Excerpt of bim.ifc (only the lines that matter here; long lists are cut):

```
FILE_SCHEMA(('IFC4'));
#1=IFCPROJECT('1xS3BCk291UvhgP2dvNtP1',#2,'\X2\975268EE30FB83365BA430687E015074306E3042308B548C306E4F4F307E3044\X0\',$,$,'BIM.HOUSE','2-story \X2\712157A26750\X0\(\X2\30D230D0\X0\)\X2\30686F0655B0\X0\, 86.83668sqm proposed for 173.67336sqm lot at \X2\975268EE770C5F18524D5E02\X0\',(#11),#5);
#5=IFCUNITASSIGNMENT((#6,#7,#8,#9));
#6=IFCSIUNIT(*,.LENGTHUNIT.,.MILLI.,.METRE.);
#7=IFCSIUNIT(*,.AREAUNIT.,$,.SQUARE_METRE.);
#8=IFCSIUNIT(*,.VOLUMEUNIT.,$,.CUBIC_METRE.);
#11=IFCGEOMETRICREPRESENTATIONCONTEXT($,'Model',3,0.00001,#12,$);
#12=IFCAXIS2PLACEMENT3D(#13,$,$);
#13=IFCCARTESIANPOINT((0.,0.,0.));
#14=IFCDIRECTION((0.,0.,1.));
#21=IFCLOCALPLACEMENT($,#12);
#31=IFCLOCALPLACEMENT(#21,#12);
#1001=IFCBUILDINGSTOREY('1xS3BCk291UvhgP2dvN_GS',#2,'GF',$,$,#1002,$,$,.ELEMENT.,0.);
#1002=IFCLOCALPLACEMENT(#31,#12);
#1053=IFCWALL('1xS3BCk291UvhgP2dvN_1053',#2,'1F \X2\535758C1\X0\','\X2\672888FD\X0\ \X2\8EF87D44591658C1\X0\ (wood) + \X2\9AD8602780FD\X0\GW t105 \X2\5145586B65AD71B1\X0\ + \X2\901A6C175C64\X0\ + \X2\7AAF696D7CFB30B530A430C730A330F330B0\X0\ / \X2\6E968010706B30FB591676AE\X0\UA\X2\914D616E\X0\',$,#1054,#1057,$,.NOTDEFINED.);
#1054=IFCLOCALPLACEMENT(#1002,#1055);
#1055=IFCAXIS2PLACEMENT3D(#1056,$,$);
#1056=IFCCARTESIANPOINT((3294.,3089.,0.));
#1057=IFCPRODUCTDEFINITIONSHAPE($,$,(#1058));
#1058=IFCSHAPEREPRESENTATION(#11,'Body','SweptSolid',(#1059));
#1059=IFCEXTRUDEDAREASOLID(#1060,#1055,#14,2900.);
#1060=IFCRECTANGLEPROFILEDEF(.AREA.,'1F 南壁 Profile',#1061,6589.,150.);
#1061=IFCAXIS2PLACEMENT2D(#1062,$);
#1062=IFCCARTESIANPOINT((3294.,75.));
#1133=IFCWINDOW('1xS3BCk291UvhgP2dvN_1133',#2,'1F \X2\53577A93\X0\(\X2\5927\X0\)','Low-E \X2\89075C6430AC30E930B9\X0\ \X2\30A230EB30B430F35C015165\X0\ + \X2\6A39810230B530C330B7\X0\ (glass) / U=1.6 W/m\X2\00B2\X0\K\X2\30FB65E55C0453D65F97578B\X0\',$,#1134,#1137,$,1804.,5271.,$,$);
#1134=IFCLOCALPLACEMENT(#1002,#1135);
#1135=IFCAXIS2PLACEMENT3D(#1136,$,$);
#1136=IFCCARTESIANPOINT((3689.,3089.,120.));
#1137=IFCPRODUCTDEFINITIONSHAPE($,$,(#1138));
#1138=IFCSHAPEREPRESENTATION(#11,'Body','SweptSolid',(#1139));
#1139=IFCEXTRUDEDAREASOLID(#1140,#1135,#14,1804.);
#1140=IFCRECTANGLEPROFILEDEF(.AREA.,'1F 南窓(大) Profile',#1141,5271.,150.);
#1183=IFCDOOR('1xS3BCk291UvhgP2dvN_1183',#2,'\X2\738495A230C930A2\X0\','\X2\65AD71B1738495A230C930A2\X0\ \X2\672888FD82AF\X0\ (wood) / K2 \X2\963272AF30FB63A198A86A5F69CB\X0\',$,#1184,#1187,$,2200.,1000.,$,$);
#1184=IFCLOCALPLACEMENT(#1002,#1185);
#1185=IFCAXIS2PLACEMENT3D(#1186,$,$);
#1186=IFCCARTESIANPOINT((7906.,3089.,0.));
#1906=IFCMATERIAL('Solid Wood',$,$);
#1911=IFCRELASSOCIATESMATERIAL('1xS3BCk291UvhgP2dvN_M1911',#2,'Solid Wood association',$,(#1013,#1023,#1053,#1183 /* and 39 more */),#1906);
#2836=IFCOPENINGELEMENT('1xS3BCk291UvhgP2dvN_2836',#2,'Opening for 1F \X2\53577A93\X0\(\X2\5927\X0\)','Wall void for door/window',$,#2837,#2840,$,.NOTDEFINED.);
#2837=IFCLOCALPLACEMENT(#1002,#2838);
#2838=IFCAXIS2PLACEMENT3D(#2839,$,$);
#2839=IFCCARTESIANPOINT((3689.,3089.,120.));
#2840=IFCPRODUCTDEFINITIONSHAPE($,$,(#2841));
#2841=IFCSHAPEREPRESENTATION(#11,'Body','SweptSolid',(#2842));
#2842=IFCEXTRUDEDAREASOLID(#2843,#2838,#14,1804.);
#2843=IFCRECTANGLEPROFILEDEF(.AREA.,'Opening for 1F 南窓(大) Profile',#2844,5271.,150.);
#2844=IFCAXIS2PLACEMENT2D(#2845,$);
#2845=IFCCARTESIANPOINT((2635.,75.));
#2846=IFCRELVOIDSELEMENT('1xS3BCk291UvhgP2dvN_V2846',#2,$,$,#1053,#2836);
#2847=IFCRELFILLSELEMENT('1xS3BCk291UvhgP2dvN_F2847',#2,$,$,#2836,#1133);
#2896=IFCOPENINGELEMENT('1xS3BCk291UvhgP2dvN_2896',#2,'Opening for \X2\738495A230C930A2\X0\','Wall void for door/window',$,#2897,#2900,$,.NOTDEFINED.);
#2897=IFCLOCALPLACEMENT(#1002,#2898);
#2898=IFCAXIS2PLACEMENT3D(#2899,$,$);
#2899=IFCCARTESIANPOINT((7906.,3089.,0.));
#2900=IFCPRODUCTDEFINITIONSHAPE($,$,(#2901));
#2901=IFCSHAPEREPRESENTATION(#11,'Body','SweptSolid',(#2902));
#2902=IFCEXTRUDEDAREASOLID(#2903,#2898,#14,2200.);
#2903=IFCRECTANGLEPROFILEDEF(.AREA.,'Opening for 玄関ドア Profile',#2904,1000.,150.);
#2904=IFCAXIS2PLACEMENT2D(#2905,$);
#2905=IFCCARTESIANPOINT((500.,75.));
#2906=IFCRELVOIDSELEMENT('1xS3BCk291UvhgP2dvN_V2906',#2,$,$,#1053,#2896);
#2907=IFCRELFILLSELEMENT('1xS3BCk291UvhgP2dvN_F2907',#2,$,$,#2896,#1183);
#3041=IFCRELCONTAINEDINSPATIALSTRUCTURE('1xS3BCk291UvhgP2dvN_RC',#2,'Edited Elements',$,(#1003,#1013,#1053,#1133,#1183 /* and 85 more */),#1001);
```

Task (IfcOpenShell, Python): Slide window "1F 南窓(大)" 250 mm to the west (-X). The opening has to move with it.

```python
import ifcopenshell
import ifcopenshell.api.geometry
import ifcopenshell.util.placement

model = ifcopenshell.open("bim.ifc")

window = model.by_guid("1xS3BCk291UvhgP2dvN_1133")
opening = window.FillsVoids[0].RelatingOpeningElement
wall = opening.VoidsElements[0].RelatingBuildingElement

wall_matrix = ifcopenshell.util.placement.get_local_placement(wall.ObjectPlacement)
shift = wall_matrix[:3, 0] * -250.0
before = ifcopenshell.util.placement.get_local_placement(window.ObjectPlacement)[:3, 3].copy()

# The window is not placed relative to its opening, so move both.
for product in (opening, window):
    matrix = ifcopenshell.util.placement.get_local_placement(product.ObjectPlacement)
    matrix[:3, 3] += shift
    ifcopenshell.api.geometry.edit_object_placement(model, product=product, matrix=matrix, is_si=False)

after = ifcopenshell.util.placement.get_local_placement(window.ObjectPlacement)[:3, 3]
print("window moved by", (after - before).round(3) + 0.0)

model.write("bim_updated.ifc")
```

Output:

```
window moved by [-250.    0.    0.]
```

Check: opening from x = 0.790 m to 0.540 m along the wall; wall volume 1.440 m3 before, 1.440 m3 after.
